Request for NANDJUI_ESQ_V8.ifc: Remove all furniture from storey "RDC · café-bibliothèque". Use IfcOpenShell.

First a look at what the model holds.

```python
import ifcopenshell
import ifcopenshell.util.element

model = ifcopenshell.open("NANDJUI_ESQ_V8.ifc")
print(model.schema)
storey = next(s for s in model.by_type("IfcBuildingStorey") if s.Name == "RDC · café-bibliothèque")
furniture = [e for e in ifcopenshell.util.element.get_decomposition(storey) if e.is_a("IfcFurnishingElement")]
seen = {}
for e in furniture:
    element_type = ifcopenshell.util.element.get_type(e)
    name = element_type.Name if element_type not in (None, e) else None
    seen[name] = seen.get(name, 0) + 1
for name, count in sorted(seen.items(), key=str):
    print(count, "x", name)
```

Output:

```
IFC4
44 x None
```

```python
import ifcopenshell
import ifcopenshell.api.root
import ifcopenshell.util.element

model = ifcopenshell.open("NANDJUI_ESQ_V8.ifc")

storey = next(s for s in model.by_type("IfcBuildingStorey") if s.Name == "RDC · café-bibliothèque")
furniture = [e for e in ifcopenshell.util.element.get_decomposition(storey) if e.is_a("IfcFurnishingElement")]

for e in furniture:
    ifcopenshell.api.root.remove_product(model, product=e)
print(len(furniture), "removed")

model.write("NANDJUI_ESQ_V8_edited.ifc")
```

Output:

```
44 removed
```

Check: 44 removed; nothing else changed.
